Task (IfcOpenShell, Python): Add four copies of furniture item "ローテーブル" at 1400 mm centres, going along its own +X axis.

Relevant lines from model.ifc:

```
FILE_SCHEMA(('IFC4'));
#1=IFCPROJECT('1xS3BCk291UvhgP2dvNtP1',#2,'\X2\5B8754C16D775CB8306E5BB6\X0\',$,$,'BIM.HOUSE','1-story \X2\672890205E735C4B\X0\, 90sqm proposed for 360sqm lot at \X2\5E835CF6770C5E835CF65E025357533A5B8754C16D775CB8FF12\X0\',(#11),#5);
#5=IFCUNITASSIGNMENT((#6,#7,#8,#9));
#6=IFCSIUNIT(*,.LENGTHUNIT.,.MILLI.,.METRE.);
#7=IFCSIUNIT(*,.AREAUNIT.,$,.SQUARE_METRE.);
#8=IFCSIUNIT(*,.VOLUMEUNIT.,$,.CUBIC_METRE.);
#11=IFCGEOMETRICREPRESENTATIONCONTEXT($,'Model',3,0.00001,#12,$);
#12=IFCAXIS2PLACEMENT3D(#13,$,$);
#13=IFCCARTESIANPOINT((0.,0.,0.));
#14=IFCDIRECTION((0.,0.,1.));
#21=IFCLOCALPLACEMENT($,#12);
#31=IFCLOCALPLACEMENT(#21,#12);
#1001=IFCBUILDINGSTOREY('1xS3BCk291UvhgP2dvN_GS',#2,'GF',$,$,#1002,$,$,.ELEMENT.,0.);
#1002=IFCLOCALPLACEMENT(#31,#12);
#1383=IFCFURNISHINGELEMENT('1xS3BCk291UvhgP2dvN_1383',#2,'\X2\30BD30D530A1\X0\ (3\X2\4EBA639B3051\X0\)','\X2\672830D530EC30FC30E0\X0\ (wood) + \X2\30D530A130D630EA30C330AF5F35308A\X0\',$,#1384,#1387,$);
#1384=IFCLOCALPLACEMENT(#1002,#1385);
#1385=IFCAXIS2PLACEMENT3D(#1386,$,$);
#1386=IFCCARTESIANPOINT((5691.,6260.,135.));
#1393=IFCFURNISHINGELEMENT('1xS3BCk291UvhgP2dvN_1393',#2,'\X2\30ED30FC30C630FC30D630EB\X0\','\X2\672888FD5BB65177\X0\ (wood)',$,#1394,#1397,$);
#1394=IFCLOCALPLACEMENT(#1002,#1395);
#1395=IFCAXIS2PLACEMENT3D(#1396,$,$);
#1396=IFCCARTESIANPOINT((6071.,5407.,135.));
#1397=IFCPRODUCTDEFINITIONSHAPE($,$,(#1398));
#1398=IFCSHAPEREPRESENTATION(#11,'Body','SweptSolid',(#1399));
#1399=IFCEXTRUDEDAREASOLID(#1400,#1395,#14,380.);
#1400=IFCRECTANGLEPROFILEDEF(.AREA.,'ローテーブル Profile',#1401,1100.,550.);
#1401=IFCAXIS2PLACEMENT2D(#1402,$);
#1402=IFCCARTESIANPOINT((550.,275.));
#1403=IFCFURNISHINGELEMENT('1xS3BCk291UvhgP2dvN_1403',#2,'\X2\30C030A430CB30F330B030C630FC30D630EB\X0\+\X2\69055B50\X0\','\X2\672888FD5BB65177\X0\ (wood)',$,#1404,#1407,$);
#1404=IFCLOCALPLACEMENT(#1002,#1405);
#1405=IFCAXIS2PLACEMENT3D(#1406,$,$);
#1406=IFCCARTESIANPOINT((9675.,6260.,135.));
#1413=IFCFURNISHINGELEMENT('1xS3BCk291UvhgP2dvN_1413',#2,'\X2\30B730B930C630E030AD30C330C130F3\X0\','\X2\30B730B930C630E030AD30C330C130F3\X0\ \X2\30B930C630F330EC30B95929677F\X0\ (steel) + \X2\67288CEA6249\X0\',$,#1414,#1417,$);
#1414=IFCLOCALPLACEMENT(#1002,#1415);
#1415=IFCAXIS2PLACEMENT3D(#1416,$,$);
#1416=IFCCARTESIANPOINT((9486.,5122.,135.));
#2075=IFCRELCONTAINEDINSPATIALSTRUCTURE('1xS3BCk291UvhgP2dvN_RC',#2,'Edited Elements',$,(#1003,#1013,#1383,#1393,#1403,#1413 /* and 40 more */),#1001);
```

```python
import ifcopenshell
import ifcopenshell.api.geometry
import ifcopenshell.api.root
import ifcopenshell.util.element
import ifcopenshell.util.placement
import ifcopenshell.util.unit

model = ifcopenshell.open("model.ifc")
unit_scale = ifcopenshell.util.unit.calculate_unit_scale(model)


def reuse_history(source, copy):
    """copy_class also copies each property set's owner history, people and application; keep the originals."""
    for rel in copy.IsDefinedBy:
        if rel.is_a("IfcRelDefinesByProperties") and (history := rel.RelatingPropertyDefinition.OwnerHistory):
            rel.RelatingPropertyDefinition.OwnerHistory = source.OwnerHistory
            ifcopenshell.util.element.remove_deep2(model, history)


source = model.by_id(1393)
base = ifcopenshell.util.placement.get_local_placement(source.ObjectPlacement)
step = base[:3, 0] * 1.4 / unit_scale

for i in range(1, 5):
    copy = ifcopenshell.api.root.copy_class(model, product=source)
    copy.Representation = ifcopenshell.util.element.copy_deep(
        model, source.Representation, exclude=["IfcGeometricRepresentationContext", "IfcRepresentationMap"]
    )
    reuse_history(source, copy)
    matrix = base.copy()
    matrix[:3, 3] += i * step
    print("added at", matrix[:3, 3].round(3) + 0.0)
    ifcopenshell.api.geometry.edit_object_placement(model, product=copy, matrix=matrix, is_si=False)

model.write("model_rev.ifc")
```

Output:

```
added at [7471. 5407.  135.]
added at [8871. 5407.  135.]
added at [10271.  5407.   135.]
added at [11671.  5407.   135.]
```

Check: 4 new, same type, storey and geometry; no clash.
